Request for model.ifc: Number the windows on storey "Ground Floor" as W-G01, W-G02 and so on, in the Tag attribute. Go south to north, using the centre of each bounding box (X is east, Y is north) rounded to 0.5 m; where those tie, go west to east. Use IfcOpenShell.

First a look at what the model holds.

```python
import ifcopenshell
import ifcopenshell.util.element
import ifcopenshell.util.placement

model = ifcopenshell.open("model.ifc")
print(model.schema)
storey = next(s for s in model.by_type("IfcBuildingStorey") if s.Name == "Ground Floor")
windows = [e for e in ifcopenshell.util.element.get_decomposition(storey) if e.is_a("IfcWindow")]
for e in sorted(windows, key=lambda e: e.id()):
    origin = ifcopenshell.util.placement.get_local_placement(e.ObjectPlacement)[:3, 3]
    print(e.id(), e.Tag, e.Name, origin.round(2) + 0.0, sep=" | ")
```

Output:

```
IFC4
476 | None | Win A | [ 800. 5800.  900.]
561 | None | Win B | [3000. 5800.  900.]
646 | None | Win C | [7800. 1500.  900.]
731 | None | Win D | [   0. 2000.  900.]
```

```python
import ifcopenshell
import ifcopenshell.geom
import ifcopenshell.util.element
import ifcopenshell.util.shape

model = ifcopenshell.open("model.ifc")
settings = ifcopenshell.geom.settings()
settings.set("use-world-coords", True)


def centre(element):
    shape = ifcopenshell.geom.create_shape(settings, element)
    return ifcopenshell.util.shape.get_bbox_centroid(shape.geometry)


storey = next(s for s in model.by_type("IfcBuildingStorey") if s.Name == "Ground Floor")
windows = [e for e in ifcopenshell.util.element.get_decomposition(storey) if e.is_a("IfcWindow")]

# Insertion points can sit at a corner or the storey origin, so sort by the geometry (in metres).
centres = {e: centre(e) for e in windows}
windows.sort(key=lambda e: (round(centres[e][1] / 0.5), centres[e][0]))

for i, e in enumerate(windows, start=1):
    number = f"W-G{i:02d}"
    e.Tag = number
    print(e.id(), number)

model.write("model_edited.ifc")
```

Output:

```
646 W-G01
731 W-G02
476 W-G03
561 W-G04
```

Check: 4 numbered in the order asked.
